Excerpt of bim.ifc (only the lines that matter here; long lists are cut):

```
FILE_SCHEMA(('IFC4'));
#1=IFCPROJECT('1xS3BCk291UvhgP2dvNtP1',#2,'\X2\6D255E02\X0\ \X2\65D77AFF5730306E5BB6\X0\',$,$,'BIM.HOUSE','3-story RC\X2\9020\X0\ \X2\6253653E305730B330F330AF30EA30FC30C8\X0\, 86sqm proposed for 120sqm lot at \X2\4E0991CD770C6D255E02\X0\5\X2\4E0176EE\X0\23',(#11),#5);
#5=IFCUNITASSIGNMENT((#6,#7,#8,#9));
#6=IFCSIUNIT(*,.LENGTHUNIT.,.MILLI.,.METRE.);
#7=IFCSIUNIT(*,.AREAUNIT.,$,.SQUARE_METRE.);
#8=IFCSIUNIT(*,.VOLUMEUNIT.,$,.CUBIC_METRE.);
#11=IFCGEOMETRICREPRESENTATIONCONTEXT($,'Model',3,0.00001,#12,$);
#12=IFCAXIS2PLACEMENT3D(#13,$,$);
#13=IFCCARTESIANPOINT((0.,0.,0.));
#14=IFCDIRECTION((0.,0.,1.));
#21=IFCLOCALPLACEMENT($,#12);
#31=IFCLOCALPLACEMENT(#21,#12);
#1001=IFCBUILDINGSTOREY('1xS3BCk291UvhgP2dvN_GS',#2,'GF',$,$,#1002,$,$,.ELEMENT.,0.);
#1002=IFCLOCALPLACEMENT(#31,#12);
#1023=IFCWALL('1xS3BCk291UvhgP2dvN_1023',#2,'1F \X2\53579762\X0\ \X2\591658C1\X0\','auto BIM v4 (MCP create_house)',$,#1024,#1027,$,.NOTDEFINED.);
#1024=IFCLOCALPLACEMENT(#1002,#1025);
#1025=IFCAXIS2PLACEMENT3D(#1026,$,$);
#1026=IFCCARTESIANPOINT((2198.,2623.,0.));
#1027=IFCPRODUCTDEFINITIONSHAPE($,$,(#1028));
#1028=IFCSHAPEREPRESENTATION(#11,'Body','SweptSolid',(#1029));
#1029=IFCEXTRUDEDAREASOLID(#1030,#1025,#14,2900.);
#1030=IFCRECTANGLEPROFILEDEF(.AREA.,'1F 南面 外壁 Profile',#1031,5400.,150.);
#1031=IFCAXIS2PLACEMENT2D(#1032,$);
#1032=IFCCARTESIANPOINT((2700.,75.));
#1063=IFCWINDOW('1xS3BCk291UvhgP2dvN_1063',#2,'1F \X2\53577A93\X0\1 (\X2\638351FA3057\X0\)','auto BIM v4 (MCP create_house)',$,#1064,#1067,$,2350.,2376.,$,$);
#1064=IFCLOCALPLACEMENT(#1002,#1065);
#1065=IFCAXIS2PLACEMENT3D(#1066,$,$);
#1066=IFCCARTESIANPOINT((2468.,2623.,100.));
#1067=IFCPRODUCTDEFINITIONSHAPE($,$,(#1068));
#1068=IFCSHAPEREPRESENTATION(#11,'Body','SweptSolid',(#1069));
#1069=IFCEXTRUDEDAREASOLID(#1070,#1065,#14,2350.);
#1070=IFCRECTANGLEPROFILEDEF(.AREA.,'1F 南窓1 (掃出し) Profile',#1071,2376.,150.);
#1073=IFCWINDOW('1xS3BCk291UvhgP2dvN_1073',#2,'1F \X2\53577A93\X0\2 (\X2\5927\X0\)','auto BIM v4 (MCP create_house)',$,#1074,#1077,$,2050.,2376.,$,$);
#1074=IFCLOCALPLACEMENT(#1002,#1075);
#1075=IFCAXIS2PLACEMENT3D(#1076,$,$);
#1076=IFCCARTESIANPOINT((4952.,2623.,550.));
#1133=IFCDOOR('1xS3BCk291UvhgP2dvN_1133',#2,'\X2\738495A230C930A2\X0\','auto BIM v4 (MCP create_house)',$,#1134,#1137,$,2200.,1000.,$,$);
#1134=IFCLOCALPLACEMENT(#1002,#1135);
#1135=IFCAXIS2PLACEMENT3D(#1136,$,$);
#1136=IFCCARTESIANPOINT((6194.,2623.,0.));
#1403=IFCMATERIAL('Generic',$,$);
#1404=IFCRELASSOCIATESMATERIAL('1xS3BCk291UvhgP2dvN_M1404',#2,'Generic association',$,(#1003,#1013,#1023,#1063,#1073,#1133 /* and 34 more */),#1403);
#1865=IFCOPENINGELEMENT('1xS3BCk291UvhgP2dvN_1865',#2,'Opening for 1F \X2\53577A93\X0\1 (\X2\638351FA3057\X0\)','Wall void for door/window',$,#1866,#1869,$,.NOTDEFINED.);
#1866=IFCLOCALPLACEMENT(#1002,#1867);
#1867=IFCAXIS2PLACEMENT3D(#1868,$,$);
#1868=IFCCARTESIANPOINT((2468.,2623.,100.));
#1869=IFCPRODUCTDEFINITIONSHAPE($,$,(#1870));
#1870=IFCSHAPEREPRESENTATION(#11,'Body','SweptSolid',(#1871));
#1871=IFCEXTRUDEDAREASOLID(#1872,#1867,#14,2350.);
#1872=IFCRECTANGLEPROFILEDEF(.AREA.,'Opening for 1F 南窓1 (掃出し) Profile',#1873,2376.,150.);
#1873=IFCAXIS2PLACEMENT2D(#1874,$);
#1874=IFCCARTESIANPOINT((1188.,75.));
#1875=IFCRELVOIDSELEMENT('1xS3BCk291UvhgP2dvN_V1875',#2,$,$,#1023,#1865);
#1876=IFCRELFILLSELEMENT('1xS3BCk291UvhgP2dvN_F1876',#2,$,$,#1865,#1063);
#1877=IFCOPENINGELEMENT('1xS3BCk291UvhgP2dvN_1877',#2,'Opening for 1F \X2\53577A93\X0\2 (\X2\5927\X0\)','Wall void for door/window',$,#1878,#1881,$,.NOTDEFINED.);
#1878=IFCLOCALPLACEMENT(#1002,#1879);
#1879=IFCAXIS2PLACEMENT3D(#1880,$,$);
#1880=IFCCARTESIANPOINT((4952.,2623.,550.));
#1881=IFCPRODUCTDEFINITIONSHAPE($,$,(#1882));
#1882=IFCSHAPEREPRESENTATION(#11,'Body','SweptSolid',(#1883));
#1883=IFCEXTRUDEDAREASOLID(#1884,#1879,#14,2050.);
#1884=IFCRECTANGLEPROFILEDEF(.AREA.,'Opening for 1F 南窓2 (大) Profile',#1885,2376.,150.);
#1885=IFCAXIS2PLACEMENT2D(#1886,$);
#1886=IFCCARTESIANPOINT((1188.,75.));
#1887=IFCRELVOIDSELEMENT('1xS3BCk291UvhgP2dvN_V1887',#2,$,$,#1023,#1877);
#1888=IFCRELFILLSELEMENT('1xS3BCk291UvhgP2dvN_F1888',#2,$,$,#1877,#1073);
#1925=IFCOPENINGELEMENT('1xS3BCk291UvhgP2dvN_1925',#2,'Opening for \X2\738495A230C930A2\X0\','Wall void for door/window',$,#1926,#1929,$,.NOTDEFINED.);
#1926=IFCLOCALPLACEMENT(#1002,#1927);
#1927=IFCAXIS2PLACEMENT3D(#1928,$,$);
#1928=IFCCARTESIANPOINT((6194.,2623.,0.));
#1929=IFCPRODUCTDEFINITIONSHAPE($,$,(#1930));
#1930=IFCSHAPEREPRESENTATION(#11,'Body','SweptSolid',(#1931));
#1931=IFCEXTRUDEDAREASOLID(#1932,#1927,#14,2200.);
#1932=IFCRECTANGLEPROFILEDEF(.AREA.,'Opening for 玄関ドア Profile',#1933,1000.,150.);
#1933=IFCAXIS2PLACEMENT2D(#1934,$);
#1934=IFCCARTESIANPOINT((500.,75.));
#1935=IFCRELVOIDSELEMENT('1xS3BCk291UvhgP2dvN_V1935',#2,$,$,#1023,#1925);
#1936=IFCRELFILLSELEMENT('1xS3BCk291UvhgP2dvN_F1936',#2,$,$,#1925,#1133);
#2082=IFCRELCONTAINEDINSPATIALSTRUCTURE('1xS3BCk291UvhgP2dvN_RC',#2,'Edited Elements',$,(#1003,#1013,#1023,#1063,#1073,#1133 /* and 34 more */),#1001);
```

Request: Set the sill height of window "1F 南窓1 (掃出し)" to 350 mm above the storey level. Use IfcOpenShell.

```python
import numpy as np
import ifcopenshell
import ifcopenshell.api.geometry
import ifcopenshell.geom
import ifcopenshell.util.element
import ifcopenshell.util.placement
import ifcopenshell.util.shape
import ifcopenshell.util.unit

model = ifcopenshell.open("bim.ifc")
unit_scale = ifcopenshell.util.unit.calculate_unit_scale(model)

window = model.by_guid("1xS3BCk291UvhgP2dvN_1063")
opening = window.FillsVoids[0].RelatingOpeningElement
storey = ifcopenshell.util.element.get_container(window, ifc_class="IfcBuildingStorey")
level = ifcopenshell.util.placement.get_local_placement(storey.ObjectPlacement)[2, 3]

# The opening's origin need not be at the sill, so measure its lowest point.
shape = ifcopenshell.geom.create_shape(ifcopenshell.geom.settings(), opening)
bottom = ifcopenshell.util.shape.get_shape_bottom_elevation(shape, shape.geometry) / unit_scale
dz = level + 0.35 / unit_scale - bottom

shift = np.array([0.0, 0.0, dz])
# The window is not placed relative to its opening, so move both.
for product in (opening, window):
    matrix = ifcopenshell.util.placement.get_local_placement(product.ObjectPlacement)
    matrix[:3, 3] += shift
    ifcopenshell.api.geometry.edit_object_placement(model, product=product, matrix=matrix, is_si=False)

print(f"moved by {dz * unit_scale:+.3f} m")

model.write("bim_edited.ifc")
```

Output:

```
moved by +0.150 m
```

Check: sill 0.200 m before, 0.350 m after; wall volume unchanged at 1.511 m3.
